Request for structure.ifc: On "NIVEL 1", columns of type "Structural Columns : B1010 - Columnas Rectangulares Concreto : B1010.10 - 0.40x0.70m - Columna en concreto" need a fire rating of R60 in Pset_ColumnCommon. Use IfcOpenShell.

First a look at what the model holds.

```python
import ifcopenshell
import ifcopenshell.util.element

model = ifcopenshell.open("structure.ifc")
print(model.schema)
storey = next(s for s in model.by_type("IfcBuildingStorey") if s.Name == "NIVEL 1")
columns = [e for e in ifcopenshell.util.element.get_decomposition(storey) if e.is_a("IfcColumn")]
seen = {}
for e in columns:
    element_type = ifcopenshell.util.element.get_type(e)
    key = (element_type.Name if element_type != e and element_type else None, ifcopenshell.util.element.get_pset(e, "Pset_ColumnCommon", "FireRating"))
    seen[key] = seen.get(key, 0) + 1
for (name, value), count in sorted(seen.items(), key=str):
    print(count, "x", name, "|", value)
```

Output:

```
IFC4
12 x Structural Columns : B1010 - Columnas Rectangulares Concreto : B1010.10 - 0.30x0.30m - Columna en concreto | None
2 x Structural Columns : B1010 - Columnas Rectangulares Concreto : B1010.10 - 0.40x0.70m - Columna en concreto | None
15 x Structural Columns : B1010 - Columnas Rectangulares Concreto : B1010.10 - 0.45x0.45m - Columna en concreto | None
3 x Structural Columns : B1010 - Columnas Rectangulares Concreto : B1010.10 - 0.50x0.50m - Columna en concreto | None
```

```python
import ifcopenshell
import ifcopenshell.api.pset
import ifcopenshell.util.element

model = ifcopenshell.open("structure.ifc")

storey = next(s for s in model.by_type("IfcBuildingStorey") if s.Name == "NIVEL 1")
columns = [e for e in ifcopenshell.util.element.get_decomposition(storey) if e.is_a("IfcColumn")]

count = 0
for e in columns:
    element_type = ifcopenshell.util.element.get_type(e)
    if element_type in (None, e) or element_type.Name != "Structural Columns : B1010 - Columnas Rectangulares Concreto : B1010.10 - 0.40x0.70m - Columna en concreto":
        continue
    # add_pset returns the element's existing set when there is one.
    pset = ifcopenshell.api.pset.add_pset(model, product=e, name="Pset_ColumnCommon")
    ifcopenshell.api.pset.edit_pset(model, pset=pset, properties={"FireRating": "R60"})
    count += 1

print(count, "columns updated")

model.write("structure_rev.ifc")
```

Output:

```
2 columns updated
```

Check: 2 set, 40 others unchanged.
